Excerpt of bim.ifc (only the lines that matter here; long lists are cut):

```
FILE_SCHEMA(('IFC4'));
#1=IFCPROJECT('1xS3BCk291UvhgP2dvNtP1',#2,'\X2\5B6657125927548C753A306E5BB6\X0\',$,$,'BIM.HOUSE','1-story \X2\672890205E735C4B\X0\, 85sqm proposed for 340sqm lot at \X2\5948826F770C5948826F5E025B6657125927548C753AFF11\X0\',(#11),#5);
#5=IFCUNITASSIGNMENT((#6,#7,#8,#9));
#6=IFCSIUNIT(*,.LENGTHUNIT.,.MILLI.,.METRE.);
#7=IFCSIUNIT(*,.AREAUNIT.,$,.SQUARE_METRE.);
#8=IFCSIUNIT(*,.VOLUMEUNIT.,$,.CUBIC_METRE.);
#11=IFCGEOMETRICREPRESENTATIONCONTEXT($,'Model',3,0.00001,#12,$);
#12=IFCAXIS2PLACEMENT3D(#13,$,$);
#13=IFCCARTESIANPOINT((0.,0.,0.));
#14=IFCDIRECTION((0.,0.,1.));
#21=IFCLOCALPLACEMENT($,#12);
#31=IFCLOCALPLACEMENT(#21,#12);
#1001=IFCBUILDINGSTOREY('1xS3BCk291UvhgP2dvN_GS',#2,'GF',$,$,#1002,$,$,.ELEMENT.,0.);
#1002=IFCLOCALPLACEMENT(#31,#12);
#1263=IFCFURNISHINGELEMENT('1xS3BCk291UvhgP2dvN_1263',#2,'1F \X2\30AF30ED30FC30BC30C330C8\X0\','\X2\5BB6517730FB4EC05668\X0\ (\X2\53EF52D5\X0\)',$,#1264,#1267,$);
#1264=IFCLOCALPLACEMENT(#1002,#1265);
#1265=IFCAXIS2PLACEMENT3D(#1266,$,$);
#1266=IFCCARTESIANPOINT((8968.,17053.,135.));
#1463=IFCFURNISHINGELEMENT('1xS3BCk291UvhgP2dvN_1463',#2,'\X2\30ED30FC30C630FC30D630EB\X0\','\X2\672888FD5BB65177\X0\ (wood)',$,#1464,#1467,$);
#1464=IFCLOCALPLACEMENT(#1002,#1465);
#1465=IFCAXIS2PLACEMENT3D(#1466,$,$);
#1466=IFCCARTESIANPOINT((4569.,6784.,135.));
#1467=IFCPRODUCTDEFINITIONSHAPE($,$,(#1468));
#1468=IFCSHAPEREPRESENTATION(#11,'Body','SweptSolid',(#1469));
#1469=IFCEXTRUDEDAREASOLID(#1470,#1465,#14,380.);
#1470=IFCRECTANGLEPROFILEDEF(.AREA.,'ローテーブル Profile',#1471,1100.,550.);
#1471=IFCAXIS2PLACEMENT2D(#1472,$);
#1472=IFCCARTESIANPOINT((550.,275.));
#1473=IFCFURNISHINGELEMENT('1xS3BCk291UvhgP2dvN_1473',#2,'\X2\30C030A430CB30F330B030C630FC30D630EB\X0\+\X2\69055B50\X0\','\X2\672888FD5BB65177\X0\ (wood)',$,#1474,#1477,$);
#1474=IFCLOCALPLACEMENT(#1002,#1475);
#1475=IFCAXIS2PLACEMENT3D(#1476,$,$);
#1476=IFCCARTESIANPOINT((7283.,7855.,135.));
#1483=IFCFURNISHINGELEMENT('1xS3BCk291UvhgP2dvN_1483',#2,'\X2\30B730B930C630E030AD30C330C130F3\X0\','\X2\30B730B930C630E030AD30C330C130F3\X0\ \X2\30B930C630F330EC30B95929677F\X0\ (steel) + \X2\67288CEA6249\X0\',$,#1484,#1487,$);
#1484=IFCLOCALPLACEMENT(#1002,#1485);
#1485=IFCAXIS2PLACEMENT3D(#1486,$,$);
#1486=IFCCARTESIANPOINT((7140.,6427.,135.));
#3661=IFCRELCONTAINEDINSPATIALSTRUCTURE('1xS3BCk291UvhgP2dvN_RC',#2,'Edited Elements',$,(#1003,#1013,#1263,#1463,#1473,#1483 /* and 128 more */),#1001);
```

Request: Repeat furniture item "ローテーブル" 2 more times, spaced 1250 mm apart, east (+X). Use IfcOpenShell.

```python
import numpy as np
import ifcopenshell
import ifcopenshell.api.geometry
import ifcopenshell.api.root
import ifcopenshell.util.element
import ifcopenshell.util.placement

model = ifcopenshell.open("bim.ifc")


def reuse_history(source, copy):
    """copy_class also copies each property set's owner history, people and application; keep the originals."""
    for rel in copy.IsDefinedBy:
        if rel.is_a("IfcRelDefinesByProperties") and (history := rel.RelatingPropertyDefinition.OwnerHistory):
            rel.RelatingPropertyDefinition.OwnerHistory = source.OwnerHistory
            ifcopenshell.util.element.remove_deep2(model, history)


source = model.by_id(1463)
base = ifcopenshell.util.placement.get_local_placement(source.ObjectPlacement)
step = np.array([1.0, 0.0, 0.0]) * 1250.0

for i in range(1, 3):
    copy = ifcopenshell.api.root.copy_class(model, product=source)
    copy.Representation = ifcopenshell.util.element.copy_deep(
        model, source.Representation, exclude=["IfcGeometricRepresentationContext", "IfcRepresentationMap"]
    )
    reuse_history(source, copy)
    matrix = base.copy()
    matrix[:3, 3] += i * step
    print("added at", matrix[:3, 3].round(3) + 0.0)
    ifcopenshell.api.geometry.edit_object_placement(model, product=copy, matrix=matrix, is_si=False)

model.write("bim_v2.ifc")
```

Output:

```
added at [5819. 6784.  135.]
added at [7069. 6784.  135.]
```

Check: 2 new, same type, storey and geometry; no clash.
